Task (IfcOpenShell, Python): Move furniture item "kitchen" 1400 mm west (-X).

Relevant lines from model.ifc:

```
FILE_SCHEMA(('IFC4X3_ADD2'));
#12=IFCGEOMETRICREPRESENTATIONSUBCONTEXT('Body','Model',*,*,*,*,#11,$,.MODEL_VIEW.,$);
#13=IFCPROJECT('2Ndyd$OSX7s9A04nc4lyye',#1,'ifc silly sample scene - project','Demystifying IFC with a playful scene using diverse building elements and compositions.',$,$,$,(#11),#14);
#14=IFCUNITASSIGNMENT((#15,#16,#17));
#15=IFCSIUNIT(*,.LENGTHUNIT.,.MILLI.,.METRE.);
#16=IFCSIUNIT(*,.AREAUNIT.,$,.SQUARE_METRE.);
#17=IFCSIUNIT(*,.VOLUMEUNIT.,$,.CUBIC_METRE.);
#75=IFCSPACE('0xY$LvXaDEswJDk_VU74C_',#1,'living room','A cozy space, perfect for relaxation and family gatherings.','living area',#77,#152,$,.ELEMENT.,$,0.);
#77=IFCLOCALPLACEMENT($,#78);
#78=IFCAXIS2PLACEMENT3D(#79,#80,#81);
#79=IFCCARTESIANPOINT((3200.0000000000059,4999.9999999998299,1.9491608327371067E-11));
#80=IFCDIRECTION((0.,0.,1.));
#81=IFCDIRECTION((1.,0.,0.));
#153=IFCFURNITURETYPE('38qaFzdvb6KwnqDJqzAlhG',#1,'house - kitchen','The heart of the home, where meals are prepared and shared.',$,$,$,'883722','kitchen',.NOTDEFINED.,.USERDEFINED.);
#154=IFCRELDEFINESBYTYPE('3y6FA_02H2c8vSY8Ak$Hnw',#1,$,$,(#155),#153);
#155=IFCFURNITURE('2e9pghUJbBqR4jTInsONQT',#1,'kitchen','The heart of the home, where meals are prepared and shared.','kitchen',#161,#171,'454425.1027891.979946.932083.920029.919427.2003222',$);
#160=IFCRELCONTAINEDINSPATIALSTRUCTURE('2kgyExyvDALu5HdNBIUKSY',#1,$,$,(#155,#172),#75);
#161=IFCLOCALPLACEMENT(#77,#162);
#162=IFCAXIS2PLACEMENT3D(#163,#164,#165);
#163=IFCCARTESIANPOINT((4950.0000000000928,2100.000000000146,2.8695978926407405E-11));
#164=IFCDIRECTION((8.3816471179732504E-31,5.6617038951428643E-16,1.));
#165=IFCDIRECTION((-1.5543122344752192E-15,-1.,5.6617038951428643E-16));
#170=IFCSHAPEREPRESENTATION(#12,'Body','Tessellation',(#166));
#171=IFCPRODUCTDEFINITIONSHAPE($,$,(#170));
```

```python
import ifcopenshell
import ifcopenshell.api.geometry
import ifcopenshell.util.placement
import ifcopenshell.util.unit

model = ifcopenshell.open("model.ifc")
unit_scale = ifcopenshell.util.unit.calculate_unit_scale(model)

item = model.by_guid("2e9pghUJbBqR4jTInsONQT")
matrix = ifcopenshell.util.placement.get_local_placement(item.ObjectPlacement)
matrix[0, 3] -= 1.4 / unit_scale
ifcopenshell.api.geometry.edit_object_placement(model, product=item, matrix=matrix, is_si=False)

print(ifcopenshell.util.placement.get_local_placement(item.ObjectPlacement).round(3) + 0.0)

model.write("model_edited.ifc")
```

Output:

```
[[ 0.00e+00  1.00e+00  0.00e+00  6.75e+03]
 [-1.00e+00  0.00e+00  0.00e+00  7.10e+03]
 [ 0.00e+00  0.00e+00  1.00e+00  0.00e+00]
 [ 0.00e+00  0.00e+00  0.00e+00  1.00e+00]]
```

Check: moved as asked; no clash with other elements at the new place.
